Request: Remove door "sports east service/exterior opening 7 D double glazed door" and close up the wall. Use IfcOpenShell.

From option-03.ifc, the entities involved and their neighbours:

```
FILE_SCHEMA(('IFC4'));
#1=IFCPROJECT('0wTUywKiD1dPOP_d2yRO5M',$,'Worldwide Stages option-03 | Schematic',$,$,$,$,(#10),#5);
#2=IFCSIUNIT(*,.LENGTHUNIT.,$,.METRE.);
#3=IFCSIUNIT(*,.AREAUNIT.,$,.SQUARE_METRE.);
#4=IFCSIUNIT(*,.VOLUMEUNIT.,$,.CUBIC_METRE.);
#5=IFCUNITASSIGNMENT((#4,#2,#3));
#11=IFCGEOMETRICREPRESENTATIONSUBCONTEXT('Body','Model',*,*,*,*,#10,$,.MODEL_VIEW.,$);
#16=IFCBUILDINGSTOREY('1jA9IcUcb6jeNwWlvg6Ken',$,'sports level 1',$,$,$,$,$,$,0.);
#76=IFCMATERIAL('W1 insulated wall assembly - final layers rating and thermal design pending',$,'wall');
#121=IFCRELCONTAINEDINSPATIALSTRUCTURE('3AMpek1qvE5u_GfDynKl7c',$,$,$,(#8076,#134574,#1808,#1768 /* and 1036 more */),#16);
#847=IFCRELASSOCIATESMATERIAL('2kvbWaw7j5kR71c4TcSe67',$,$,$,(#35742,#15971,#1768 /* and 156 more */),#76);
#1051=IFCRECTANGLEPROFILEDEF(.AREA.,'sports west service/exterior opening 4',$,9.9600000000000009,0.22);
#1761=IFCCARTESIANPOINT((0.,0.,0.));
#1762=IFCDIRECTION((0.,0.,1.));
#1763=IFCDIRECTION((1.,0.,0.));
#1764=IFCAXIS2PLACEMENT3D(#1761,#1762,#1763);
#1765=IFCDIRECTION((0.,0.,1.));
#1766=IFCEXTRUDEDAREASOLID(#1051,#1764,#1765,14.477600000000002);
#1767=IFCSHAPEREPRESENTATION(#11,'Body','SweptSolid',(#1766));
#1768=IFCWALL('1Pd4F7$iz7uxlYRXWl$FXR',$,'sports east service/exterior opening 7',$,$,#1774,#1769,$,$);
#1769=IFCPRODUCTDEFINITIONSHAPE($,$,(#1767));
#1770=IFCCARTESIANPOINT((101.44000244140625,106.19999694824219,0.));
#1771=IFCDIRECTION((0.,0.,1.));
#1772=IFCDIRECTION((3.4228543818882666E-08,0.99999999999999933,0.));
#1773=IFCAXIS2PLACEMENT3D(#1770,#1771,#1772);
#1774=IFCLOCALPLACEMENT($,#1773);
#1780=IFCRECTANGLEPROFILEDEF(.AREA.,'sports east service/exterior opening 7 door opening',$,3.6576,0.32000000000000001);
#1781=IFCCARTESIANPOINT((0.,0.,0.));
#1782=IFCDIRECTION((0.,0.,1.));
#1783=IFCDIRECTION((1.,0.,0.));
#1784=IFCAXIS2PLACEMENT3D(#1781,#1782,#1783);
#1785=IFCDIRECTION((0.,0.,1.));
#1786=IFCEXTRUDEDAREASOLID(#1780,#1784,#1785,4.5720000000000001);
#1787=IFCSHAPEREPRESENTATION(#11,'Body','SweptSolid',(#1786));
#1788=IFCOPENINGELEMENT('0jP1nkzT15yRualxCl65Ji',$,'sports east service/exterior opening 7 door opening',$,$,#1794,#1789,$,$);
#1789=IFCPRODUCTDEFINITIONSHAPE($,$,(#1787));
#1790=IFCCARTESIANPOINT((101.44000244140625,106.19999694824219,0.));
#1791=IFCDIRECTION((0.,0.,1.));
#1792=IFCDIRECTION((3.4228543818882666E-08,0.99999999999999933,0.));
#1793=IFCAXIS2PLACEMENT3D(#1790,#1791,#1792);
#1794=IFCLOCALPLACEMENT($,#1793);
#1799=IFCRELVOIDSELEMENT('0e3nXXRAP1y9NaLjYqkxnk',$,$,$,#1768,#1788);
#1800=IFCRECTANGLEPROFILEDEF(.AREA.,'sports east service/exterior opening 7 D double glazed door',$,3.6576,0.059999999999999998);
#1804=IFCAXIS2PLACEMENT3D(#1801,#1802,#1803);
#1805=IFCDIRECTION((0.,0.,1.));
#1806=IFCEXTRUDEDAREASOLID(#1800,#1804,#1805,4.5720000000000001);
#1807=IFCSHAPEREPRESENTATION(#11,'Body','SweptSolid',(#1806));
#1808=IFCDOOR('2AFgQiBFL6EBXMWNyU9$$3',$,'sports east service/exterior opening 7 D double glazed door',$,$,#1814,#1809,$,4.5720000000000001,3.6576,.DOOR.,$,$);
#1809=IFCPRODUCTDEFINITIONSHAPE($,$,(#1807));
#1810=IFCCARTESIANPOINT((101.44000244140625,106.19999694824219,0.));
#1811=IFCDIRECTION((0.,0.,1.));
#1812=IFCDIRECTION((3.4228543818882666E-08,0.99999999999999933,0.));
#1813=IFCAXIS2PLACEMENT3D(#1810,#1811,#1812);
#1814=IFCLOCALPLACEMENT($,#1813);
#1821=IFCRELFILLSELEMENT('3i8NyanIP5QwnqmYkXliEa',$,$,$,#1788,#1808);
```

```python
import ifcopenshell
import ifcopenshell.api.feature
import ifcopenshell.api.root
import ifcopenshell.geom
import ifcopenshell.util.shape

model = ifcopenshell.open("option-03.ifc")
settings = ifcopenshell.geom.settings()


def volume(element):
    """Net volume in cubic metres, openings subtracted."""
    shape = ifcopenshell.geom.create_shape(settings, element)
    return ifcopenshell.util.shape.get_volume(shape.geometry)


door = model.by_guid("2AFgQiBFL6EBXMWNyU9$$3")
opening = door.FillsVoids[0].RelatingOpeningElement
wall = opening.VoidsElements[0].RelatingBuildingElement
before = volume(wall)

ifcopenshell.api.root.remove_product(model, product=door)
ifcopenshell.api.feature.remove_feature(model, feature=opening)

after = volume(wall)

print(f"wall volume {before:.3f} -> {after:.3f} m3")

model.write("option-03_rev.ifc")
```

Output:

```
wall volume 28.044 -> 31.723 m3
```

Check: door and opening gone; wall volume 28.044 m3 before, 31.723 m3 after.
